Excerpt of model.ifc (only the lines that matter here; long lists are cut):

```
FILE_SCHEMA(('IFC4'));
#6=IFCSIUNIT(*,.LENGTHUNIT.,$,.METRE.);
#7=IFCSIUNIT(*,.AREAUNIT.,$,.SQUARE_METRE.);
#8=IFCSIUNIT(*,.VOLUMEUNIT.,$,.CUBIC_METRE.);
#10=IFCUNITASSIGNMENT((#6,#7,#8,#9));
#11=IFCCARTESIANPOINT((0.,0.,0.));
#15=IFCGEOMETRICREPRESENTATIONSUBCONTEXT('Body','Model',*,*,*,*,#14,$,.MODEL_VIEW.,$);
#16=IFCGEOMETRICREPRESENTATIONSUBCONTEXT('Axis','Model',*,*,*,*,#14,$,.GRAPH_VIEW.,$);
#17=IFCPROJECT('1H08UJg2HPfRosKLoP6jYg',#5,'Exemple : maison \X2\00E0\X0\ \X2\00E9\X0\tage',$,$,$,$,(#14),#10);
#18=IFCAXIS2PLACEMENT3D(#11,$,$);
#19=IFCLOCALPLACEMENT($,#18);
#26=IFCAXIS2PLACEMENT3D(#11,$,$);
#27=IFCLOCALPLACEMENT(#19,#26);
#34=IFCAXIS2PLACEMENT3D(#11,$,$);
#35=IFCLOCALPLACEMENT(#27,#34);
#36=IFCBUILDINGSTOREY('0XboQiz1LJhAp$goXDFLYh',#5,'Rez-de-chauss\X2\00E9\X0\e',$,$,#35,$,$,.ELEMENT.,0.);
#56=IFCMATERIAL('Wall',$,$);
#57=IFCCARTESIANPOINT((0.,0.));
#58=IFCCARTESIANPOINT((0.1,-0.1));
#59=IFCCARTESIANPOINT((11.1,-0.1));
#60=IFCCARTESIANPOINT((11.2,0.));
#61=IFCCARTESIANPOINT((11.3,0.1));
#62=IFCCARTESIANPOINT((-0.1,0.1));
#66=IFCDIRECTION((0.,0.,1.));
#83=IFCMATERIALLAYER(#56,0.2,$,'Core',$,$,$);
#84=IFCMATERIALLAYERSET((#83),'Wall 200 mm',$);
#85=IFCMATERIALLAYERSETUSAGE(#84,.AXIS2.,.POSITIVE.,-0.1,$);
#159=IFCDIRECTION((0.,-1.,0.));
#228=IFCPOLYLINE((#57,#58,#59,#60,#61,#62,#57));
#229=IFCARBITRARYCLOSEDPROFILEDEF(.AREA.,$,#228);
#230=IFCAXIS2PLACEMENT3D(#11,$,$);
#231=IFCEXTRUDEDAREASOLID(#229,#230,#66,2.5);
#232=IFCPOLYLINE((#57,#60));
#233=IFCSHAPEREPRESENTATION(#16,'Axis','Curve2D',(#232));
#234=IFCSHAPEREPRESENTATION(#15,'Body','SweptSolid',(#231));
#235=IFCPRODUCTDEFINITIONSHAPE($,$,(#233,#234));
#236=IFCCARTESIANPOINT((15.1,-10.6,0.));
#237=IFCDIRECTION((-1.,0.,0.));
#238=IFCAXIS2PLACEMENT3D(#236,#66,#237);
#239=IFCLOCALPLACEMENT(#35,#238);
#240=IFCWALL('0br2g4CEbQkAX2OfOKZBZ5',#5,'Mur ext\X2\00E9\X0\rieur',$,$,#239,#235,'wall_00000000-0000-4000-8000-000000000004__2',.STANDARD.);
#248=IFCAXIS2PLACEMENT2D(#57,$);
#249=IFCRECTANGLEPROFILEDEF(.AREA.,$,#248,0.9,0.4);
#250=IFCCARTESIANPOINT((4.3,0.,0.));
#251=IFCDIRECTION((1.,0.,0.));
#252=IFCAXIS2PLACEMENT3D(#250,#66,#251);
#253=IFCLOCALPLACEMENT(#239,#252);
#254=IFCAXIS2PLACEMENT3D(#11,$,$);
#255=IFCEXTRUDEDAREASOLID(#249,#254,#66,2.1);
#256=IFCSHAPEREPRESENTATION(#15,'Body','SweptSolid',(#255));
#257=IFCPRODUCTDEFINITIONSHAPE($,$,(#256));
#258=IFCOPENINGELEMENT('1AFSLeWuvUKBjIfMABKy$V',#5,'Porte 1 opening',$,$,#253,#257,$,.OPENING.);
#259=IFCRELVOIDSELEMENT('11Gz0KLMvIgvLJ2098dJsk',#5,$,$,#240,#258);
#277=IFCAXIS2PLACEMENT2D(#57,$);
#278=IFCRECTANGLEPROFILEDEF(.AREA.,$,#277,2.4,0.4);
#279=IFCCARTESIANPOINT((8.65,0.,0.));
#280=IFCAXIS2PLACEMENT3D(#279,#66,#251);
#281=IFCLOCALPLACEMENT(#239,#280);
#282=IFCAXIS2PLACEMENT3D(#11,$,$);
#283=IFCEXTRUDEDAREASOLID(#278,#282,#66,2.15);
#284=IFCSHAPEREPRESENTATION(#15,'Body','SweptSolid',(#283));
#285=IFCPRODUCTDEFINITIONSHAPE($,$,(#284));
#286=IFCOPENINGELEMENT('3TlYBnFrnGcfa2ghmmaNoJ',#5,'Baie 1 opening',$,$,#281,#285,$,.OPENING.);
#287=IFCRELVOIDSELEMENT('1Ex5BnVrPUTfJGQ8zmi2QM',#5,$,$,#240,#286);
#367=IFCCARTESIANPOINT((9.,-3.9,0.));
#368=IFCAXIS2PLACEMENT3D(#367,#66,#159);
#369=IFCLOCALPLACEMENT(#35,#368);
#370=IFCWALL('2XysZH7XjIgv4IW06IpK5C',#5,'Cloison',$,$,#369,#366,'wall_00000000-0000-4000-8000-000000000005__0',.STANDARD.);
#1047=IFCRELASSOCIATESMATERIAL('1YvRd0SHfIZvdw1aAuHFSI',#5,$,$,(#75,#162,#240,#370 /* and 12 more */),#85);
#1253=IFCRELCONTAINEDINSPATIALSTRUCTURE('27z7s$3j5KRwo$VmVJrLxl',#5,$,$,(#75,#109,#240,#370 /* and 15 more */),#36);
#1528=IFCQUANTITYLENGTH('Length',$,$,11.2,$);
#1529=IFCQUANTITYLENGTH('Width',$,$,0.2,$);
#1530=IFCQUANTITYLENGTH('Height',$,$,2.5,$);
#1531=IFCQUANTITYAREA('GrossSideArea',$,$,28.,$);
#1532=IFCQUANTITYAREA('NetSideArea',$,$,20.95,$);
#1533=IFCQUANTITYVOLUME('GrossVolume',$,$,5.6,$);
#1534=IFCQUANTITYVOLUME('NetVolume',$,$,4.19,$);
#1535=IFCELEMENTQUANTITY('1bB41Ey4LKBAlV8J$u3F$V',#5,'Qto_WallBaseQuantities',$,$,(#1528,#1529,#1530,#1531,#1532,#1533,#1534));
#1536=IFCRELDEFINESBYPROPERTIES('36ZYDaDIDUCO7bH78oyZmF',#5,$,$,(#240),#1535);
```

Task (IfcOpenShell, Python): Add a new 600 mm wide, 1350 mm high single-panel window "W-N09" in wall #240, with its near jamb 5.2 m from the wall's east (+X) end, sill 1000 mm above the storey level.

```python
import numpy as np
import ifcopenshell
import ifcopenshell.api.feature
import ifcopenshell.api.geometry
import ifcopenshell.api.pset
import ifcopenshell.api.root
import ifcopenshell.api.spatial
import ifcopenshell.geom
import ifcopenshell.util.element
import ifcopenshell.util.placement
import ifcopenshell.util.representation
import ifcopenshell.util.shape
import ifcopenshell.util.unit

model = ifcopenshell.open("model.ifc")
unit_scale = ifcopenshell.util.unit.calculate_unit_scale(model)
area_scale = ifcopenshell.util.unit.calculate_unit_scale(model, "AREAUNIT")
volume_scale = ifcopenshell.util.unit.calculate_unit_scale(model, "VOLUMEUNIT")
settings = ifcopenshell.geom.settings()


def volume(element):
    """Net volume in cubic metres, openings subtracted."""
    shape = ifcopenshell.geom.create_shape(settings, element)
    return ifcopenshell.util.shape.get_volume(shape.geometry)


wall = model.by_guid("0br2g4CEbQkAX2OfOKZBZ5")
storey = ifcopenshell.util.element.get_container(wall, ifc_class="IfcBuildingStorey")
context = ifcopenshell.util.representation.get_context(model, "Model", "Body", "MODEL_VIEW")
before = volume(wall)

width, height, from_end, sill = 0.6, 1.35, 5.2, 1  # metres

# The wall runs along its own X axis, and the end named is its -X end.
wall_shape = ifcopenshell.geom.create_shape(settings, wall)
x, y, z = ifcopenshell.util.shape.get_vertices(wall_shape.geometry).T
start = x.min() + from_end
face, thickness = float(y.min()), float(y.max() - y.min())
wall_matrix = ifcopenshell.util.placement.get_local_placement(wall.ObjectPlacement)
level = ifcopenshell.util.placement.get_local_placement(storey.ObjectPlacement)[2, 3]


def in_wall(x, y):
    """Placement at x, y metres in the wall's axes, at sill height."""
    matrix = wall_matrix.copy()
    matrix[:, 3] = wall_matrix @ np.array([x / unit_scale, y / unit_scale, 0.0, 1.0])
    matrix[2, 3] = level + sill / unit_scale
    return matrix


# Opening: a box that overshoots both wall faces by 50 mm.
opening = ifcopenshell.api.root.create_entity(model, ifc_class="IfcOpeningElement", predefined_type="OPENING")
box = ifcopenshell.api.geometry.add_wall_representation(
    model, context=context, length=width, height=height, thickness=thickness + 0.1
)
ifcopenshell.api.geometry.assign_representation(model, product=opening, representation=box)
ifcopenshell.api.geometry.edit_object_placement(model, product=opening, matrix=in_wall(start, face - 0.05), is_si=False)
ifcopenshell.api.feature.add_feature(model, feature=opening, element=wall)

window = ifcopenshell.api.root.create_entity(model, ifc_class="IfcWindow", name="W-N09", predefined_type="WINDOW")
window.OverallWidth, window.OverallHeight = width / unit_scale, height / unit_scale
window.PartitioningType = "SINGLE_PANEL"
body = ifcopenshell.api.geometry.add_window_representation(
    model,
    context=context,
    overall_width=window.OverallWidth,
    overall_height=window.OverallHeight,
    partition_type="SINGLE_PANEL",
)
ifcopenshell.api.geometry.assign_representation(model, product=window, representation=body)
ifcopenshell.api.spatial.assign_container(model, products=[window], relating_structure=storey)
ifcopenshell.api.feature.add_filling(model, opening=opening, element=window)

# Centre the window in the wall's thickness.
ifcopenshell.api.geometry.edit_object_placement(model, product=window, matrix=in_wall(start, face), is_si=False)
window_shape = ifcopenshell.geom.create_shape(settings, window)
depth = ifcopenshell.util.shape.get_vertices(window_shape.geometry)[:, 1]
offset = face + thickness / 2 - (depth.min() + depth.max()) / 2
ifcopenshell.api.geometry.edit_object_placement(model, product=window, matrix=in_wall(start, offset), is_si=False)

after = volume(wall)

# Update the wall's stored quantities.
qto = model.by_id(ifcopenshell.util.element.get_pset(wall, "Qto_WallBaseQuantities", should_inherit=False)["id"])
ifcopenshell.api.pset.edit_qto(model, qto=qto, properties={
    "NetSideArea": after / thickness / area_scale,
    "NetVolume": after / volume_scale,
})

print(f"wall volume {before:.3f} -> {after:.3f} m3")

model.write("model_updated.ifc")
```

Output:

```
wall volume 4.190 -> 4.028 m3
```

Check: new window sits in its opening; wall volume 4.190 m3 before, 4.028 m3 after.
